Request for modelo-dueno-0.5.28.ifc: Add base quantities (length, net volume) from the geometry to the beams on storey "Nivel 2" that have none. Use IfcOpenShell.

First a look at what the model holds.

```python
import ifcopenshell
import ifcopenshell.util.element
import ifcopenshell.util.unit

model = ifcopenshell.open("modelo-dueno-0.5.28.ifc")
print(model.schema)
for unit_type in ("LENGTHUNIT", "AREAUNIT", "VOLUMEUNIT"):
    print(unit_type, ifcopenshell.util.unit.calculate_unit_scale(model, unit_type))
storey = next(s for s in model.by_type("IfcBuildingStorey") if s.Name == "Nivel 2")
beams = [e for e in ifcopenshell.util.element.get_decomposition(storey) if e.is_a("IfcBeam")]
for e in sorted(beams, key=lambda e: e.id()):
    print(e.id(), e.is_a(), e.Name, list(ifcopenshell.util.element.get_psets(e, qtos_only=True)), sep=" | ")
```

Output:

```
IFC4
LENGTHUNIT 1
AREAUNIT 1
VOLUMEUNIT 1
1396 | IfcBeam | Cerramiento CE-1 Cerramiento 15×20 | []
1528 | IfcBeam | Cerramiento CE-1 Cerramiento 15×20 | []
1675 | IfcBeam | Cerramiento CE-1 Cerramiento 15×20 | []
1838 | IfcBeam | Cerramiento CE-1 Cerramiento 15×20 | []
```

```python
import ifcopenshell
import ifcopenshell.api.pset
import ifcopenshell.geom
import ifcopenshell.util.element
import ifcopenshell.util.shape
import ifcopenshell.util.unit

model = ifcopenshell.open("modelo-dueno-0.5.28.ifc")
unit_scale = ifcopenshell.util.unit.calculate_unit_scale(model)
volume_scale = ifcopenshell.util.unit.calculate_unit_scale(model, "VOLUMEUNIT")
settings = ifcopenshell.geom.settings()

storey = next(s for s in model.by_type("IfcBuildingStorey") if s.Name == "Nivel 2")
beams = [e for e in ifcopenshell.util.element.get_decomposition(storey) if e.is_a("IfcBeam")]

for e in sorted(beams, key=lambda e: e.id()):
    if ifcopenshell.util.element.get_psets(e, qtos_only=True, should_inherit=False):
        continue
    # Geometry comes back in metres, in the element's own axes.
    shape = ifcopenshell.geom.create_shape(settings, e)
    values = {
        "Length": ifcopenshell.util.shape.get_max_xyz(shape.geometry) / unit_scale,
        "NetVolume": ifcopenshell.util.shape.get_volume(shape.geometry) / volume_scale,
    }
    qto = ifcopenshell.api.pset.add_qto(model, product=e, name="Qto_BeamBaseQuantities")
    ifcopenshell.api.pset.edit_qto(model, qto=qto, properties=values)
    print(e.id(), {k: round(v, 3) for k, v in values.items()})

model.write("modelo-dueno-0.5.28_edited.ifc")
```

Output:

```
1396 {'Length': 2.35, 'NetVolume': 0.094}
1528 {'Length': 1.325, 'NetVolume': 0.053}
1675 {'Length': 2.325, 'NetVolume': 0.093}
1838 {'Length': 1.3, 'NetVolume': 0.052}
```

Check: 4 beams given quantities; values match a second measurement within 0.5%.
